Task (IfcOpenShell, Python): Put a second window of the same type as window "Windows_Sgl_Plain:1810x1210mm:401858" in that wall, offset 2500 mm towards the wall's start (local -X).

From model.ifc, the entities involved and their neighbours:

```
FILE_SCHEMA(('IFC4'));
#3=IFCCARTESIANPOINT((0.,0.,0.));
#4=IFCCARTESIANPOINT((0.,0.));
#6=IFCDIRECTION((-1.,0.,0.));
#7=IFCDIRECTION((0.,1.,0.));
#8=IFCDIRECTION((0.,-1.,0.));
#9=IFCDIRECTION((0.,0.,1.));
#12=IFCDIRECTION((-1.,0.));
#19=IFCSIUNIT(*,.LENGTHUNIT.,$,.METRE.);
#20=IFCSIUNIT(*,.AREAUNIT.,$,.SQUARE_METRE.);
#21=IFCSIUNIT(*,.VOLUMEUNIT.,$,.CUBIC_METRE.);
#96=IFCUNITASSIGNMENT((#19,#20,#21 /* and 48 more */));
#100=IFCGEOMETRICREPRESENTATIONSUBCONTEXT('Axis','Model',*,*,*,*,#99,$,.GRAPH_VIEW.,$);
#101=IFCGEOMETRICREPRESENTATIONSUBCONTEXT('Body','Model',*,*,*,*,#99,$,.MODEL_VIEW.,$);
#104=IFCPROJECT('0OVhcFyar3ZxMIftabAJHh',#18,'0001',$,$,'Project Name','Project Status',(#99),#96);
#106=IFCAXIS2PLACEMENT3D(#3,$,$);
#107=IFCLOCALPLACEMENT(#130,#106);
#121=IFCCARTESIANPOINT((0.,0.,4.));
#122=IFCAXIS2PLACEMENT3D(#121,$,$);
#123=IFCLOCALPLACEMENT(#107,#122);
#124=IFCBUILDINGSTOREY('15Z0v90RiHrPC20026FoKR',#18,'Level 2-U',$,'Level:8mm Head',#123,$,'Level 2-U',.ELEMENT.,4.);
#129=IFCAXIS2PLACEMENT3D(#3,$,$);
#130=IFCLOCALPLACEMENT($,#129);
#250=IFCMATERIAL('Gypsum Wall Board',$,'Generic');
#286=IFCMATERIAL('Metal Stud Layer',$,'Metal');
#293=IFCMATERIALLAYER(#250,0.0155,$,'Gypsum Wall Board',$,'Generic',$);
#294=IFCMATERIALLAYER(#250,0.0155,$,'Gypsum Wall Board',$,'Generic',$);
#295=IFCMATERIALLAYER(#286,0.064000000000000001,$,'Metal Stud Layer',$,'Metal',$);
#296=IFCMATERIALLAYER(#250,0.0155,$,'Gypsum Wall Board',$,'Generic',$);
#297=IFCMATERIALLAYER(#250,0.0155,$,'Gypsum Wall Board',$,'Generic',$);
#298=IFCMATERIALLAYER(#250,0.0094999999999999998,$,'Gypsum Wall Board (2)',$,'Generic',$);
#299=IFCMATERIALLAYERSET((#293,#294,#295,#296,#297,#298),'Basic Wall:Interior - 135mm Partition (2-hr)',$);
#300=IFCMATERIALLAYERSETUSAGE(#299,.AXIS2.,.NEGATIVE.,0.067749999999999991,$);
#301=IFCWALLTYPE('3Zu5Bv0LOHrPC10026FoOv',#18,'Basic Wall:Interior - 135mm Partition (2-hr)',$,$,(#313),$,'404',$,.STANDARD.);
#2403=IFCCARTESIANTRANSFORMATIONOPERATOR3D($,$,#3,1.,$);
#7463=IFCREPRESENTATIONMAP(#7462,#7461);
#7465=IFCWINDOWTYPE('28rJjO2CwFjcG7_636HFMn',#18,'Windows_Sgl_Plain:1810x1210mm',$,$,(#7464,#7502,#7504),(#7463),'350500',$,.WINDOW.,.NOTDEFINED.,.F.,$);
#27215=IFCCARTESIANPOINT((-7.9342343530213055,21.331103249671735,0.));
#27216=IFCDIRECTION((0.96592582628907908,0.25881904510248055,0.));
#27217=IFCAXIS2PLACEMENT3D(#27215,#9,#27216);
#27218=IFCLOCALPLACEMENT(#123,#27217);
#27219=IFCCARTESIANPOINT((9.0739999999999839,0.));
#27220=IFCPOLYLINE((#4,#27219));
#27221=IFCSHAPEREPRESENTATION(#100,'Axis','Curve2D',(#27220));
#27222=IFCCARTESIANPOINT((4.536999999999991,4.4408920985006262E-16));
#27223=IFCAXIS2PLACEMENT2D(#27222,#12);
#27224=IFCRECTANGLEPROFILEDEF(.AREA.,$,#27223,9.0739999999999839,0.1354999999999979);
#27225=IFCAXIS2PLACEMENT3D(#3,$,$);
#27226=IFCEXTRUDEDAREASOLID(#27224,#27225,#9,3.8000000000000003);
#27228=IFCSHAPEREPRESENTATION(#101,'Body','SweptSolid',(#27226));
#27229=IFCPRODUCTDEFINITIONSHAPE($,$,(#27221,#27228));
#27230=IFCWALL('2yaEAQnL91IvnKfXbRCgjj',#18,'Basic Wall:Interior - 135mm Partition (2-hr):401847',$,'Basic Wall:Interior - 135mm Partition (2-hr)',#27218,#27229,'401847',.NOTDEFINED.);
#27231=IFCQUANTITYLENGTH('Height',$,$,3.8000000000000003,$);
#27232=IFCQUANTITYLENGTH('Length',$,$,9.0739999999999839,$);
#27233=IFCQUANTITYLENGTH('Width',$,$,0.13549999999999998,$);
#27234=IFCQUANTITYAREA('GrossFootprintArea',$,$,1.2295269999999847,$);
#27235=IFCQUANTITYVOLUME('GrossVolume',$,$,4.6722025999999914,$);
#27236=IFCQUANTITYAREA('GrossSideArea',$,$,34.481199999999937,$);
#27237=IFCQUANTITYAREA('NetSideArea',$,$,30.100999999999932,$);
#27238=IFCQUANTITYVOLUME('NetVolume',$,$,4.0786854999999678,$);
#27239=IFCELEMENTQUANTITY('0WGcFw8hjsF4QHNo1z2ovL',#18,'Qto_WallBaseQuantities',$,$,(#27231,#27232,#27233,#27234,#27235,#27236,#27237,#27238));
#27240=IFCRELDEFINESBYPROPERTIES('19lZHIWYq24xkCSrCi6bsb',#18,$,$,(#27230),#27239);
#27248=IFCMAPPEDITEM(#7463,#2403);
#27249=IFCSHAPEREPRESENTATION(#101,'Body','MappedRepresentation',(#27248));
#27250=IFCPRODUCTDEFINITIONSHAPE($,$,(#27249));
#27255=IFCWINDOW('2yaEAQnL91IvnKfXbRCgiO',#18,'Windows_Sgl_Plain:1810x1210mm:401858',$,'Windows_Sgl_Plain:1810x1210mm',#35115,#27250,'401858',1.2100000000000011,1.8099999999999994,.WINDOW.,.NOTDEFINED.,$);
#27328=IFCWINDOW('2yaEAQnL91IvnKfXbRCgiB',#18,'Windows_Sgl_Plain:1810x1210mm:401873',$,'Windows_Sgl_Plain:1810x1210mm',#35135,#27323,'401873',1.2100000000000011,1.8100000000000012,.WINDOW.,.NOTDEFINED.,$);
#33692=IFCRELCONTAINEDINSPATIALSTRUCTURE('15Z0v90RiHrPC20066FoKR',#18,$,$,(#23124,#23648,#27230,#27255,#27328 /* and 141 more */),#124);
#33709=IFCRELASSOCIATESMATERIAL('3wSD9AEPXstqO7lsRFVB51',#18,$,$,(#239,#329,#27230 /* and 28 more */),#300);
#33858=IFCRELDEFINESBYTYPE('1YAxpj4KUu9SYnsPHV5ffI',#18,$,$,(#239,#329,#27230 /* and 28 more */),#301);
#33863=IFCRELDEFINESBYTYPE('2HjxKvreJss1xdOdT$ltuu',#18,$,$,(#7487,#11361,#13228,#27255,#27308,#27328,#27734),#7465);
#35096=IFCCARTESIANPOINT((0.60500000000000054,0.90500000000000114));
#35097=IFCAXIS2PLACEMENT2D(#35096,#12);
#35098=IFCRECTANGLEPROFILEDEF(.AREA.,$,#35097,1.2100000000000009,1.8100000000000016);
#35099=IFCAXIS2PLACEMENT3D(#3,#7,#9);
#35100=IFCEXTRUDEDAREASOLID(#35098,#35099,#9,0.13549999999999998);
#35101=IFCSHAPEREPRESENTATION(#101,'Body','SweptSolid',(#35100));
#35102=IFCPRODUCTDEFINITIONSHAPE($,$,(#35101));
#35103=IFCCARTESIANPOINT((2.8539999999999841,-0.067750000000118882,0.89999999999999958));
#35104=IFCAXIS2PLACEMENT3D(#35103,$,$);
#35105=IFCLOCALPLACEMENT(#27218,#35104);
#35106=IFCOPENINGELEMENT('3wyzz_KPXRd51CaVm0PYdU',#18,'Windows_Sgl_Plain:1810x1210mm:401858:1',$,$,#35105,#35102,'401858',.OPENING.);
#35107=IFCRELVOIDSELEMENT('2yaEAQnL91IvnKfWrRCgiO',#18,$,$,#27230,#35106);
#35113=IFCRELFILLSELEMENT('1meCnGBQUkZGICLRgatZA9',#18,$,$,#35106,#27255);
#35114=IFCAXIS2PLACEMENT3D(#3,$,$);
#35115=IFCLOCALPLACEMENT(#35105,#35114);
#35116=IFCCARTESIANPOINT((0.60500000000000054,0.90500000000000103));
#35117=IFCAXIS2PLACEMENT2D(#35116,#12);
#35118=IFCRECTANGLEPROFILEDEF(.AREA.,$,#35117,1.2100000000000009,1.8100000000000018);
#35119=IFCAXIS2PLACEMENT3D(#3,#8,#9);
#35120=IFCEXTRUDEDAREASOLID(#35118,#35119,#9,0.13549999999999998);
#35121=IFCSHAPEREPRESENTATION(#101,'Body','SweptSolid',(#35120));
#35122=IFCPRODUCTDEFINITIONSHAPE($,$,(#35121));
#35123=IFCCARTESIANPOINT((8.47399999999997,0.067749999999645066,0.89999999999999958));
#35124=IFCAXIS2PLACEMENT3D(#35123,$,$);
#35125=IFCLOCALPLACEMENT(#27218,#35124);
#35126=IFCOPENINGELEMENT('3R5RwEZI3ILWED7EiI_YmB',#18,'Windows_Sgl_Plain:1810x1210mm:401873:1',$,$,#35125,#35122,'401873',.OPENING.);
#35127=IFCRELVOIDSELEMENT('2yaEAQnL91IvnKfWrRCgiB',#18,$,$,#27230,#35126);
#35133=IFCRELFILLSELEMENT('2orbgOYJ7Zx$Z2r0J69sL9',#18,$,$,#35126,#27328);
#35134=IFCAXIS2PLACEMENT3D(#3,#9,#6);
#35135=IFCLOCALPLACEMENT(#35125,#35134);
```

```python
import ifcopenshell
import ifcopenshell.api.feature
import ifcopenshell.api.geometry
import ifcopenshell.api.pset
import ifcopenshell.api.root
import ifcopenshell.geom
import ifcopenshell.util.element
import ifcopenshell.util.placement
import ifcopenshell.util.shape
import ifcopenshell.util.unit

model = ifcopenshell.open("model.ifc")
area_scale = ifcopenshell.util.unit.calculate_unit_scale(model, "AREAUNIT")
volume_scale = ifcopenshell.util.unit.calculate_unit_scale(model, "VOLUMEUNIT")
settings = ifcopenshell.geom.settings()


def volume(element):
    """Net volume in cubic metres, openings subtracted."""
    shape = ifcopenshell.geom.create_shape(settings, element)
    return ifcopenshell.util.shape.get_volume(shape.geometry)


def reuse_history(source, copy):
    """copy_class also copies each property set's owner history, people and application; keep the originals."""
    for rel in copy.IsDefinedBy:
        if rel.is_a("IfcRelDefinesByProperties") and (history := rel.RelatingPropertyDefinition.OwnerHistory):
            rel.RelatingPropertyDefinition.OwnerHistory = source.OwnerHistory
            ifcopenshell.util.element.remove_deep2(model, history)


window = model.by_guid("2yaEAQnL91IvnKfXbRCgiO")
opening = window.FillsVoids[0].RelatingOpeningElement
wall = opening.VoidsElements[0].RelatingBuildingElement
before = volume(wall)
shift = ifcopenshell.util.placement.get_local_placement(wall.ObjectPlacement)[:3, 0] * -2.5

# copy_class copies the void relationship, type, container and properties, but no geometry.
new_opening = ifcopenshell.api.root.copy_class(model, product=opening)
new_opening.Representation = ifcopenshell.util.element.copy_deep(
    model, opening.Representation, exclude=["IfcGeometricRepresentationContext", "IfcRepresentationMap"]
)
new_opening.Name = "Windows_Sgl_Plain:1810x1210mm"
new_opening.Tag = None
reuse_history(opening, new_opening)
new_window = ifcopenshell.api.root.copy_class(model, product=window)
new_window.Representation = ifcopenshell.util.element.copy_deep(
    model, window.Representation, exclude=["IfcGeometricRepresentationContext", "IfcRepresentationMap"]
)
new_window.Name = "Windows_Sgl_Plain:1810x1210mm"
new_window.Tag = None
reuse_history(window, new_window)
ifcopenshell.api.feature.add_filling(model, opening=new_opening, element=new_window)

for old, new in ((opening, new_opening), (window, new_window)):
    matrix = ifcopenshell.util.placement.get_local_placement(old.ObjectPlacement)
    matrix[:3, 3] += shift
    ifcopenshell.api.geometry.edit_object_placement(model, product=new, matrix=matrix, is_si=False)

after = volume(wall)
thickness = 0.1355  # wall thickness in metres

# Update the wall's stored quantities.
qto = model.by_id(ifcopenshell.util.element.get_pset(wall, "Qto_WallBaseQuantities", should_inherit=False)["id"])
ifcopenshell.api.pset.edit_qto(model, qto=qto, properties={
    "NetSideArea": after / thickness / area_scale,
    "NetVolume": after / volume_scale,
})

print(f"wall volume {before:.3f} -> {after:.3f} m3")

model.write("model_edited.ifc")
```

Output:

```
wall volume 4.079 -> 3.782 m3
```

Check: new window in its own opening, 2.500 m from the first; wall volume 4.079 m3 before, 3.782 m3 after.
